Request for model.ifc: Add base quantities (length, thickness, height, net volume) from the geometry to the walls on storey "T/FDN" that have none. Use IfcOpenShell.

First a look at what the model holds.

```python
import ifcopenshell
import ifcopenshell.util.element
import ifcopenshell.util.unit

model = ifcopenshell.open("model.ifc")
print(model.schema)
for unit_type in ("LENGTHUNIT", "AREAUNIT", "VOLUMEUNIT"):
    print(unit_type, ifcopenshell.util.unit.calculate_unit_scale(model, unit_type))
storey = next(s for s in model.by_type("IfcBuildingStorey") if s.Name == "T/FDN")
walls = [e for e in ifcopenshell.util.element.get_decomposition(storey) if e.is_a("IfcWall")]
for e in sorted(walls, key=lambda e: e.id()):
    print(e.id(), e.is_a(), e.Name, list(ifcopenshell.util.element.get_psets(e, qtos_only=True)), sep=" | ")
```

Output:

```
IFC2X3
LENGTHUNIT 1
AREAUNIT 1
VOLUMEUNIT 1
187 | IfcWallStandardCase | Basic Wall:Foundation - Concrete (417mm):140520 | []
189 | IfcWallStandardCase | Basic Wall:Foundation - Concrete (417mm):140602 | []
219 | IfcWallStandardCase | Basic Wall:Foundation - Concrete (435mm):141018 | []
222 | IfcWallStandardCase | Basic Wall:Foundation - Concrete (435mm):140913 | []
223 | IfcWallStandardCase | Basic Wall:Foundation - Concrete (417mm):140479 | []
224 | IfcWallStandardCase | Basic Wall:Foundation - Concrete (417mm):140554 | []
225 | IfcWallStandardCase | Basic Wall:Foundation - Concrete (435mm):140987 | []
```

```python
import ifcopenshell
import ifcopenshell.api.pset
import ifcopenshell.geom
import ifcopenshell.util.element
import ifcopenshell.util.shape
import ifcopenshell.util.unit

model = ifcopenshell.open("model.ifc")
unit_scale = ifcopenshell.util.unit.calculate_unit_scale(model)
volume_scale = ifcopenshell.util.unit.calculate_unit_scale(model, "VOLUMEUNIT")
settings = ifcopenshell.geom.settings()

storey = next(s for s in model.by_type("IfcBuildingStorey") if s.Name == "T/FDN")
walls = [e for e in ifcopenshell.util.element.get_decomposition(storey) if e.is_a("IfcWall")]

for e in sorted(walls, key=lambda e: e.id()):
    if ifcopenshell.util.element.get_psets(e, qtos_only=True, should_inherit=False):
        continue
    # Geometry comes back in metres, in the element's own axes.
    shape = ifcopenshell.geom.create_shape(settings, e)
    values = {
        "Length": ifcopenshell.util.shape.get_x(shape.geometry) / unit_scale,
        "Width": ifcopenshell.util.shape.get_y(shape.geometry) / unit_scale,
        "Height": ifcopenshell.util.shape.get_z(shape.geometry) / unit_scale,
        "NetVolume": ifcopenshell.util.shape.get_volume(shape.geometry) / volume_scale,
    }
    qto = ifcopenshell.api.pset.add_qto(model, product=e, name="BaseQuantities")
    ifcopenshell.api.pset.edit_qto(model, qto=qto, properties=values)
    print(e.id(), {k: round(v, 3) for k, v in values.items()})

model.write("model-out.ifc")
```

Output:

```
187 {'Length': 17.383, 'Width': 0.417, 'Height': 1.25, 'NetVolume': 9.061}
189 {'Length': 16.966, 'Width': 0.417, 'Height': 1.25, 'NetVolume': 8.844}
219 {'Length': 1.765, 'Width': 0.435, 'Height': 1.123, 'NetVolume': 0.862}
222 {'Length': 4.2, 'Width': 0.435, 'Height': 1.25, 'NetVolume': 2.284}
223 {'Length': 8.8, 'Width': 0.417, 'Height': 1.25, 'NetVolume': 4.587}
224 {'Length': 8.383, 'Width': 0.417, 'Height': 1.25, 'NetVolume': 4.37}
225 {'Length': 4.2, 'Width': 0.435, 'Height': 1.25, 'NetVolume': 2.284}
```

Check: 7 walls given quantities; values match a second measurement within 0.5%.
